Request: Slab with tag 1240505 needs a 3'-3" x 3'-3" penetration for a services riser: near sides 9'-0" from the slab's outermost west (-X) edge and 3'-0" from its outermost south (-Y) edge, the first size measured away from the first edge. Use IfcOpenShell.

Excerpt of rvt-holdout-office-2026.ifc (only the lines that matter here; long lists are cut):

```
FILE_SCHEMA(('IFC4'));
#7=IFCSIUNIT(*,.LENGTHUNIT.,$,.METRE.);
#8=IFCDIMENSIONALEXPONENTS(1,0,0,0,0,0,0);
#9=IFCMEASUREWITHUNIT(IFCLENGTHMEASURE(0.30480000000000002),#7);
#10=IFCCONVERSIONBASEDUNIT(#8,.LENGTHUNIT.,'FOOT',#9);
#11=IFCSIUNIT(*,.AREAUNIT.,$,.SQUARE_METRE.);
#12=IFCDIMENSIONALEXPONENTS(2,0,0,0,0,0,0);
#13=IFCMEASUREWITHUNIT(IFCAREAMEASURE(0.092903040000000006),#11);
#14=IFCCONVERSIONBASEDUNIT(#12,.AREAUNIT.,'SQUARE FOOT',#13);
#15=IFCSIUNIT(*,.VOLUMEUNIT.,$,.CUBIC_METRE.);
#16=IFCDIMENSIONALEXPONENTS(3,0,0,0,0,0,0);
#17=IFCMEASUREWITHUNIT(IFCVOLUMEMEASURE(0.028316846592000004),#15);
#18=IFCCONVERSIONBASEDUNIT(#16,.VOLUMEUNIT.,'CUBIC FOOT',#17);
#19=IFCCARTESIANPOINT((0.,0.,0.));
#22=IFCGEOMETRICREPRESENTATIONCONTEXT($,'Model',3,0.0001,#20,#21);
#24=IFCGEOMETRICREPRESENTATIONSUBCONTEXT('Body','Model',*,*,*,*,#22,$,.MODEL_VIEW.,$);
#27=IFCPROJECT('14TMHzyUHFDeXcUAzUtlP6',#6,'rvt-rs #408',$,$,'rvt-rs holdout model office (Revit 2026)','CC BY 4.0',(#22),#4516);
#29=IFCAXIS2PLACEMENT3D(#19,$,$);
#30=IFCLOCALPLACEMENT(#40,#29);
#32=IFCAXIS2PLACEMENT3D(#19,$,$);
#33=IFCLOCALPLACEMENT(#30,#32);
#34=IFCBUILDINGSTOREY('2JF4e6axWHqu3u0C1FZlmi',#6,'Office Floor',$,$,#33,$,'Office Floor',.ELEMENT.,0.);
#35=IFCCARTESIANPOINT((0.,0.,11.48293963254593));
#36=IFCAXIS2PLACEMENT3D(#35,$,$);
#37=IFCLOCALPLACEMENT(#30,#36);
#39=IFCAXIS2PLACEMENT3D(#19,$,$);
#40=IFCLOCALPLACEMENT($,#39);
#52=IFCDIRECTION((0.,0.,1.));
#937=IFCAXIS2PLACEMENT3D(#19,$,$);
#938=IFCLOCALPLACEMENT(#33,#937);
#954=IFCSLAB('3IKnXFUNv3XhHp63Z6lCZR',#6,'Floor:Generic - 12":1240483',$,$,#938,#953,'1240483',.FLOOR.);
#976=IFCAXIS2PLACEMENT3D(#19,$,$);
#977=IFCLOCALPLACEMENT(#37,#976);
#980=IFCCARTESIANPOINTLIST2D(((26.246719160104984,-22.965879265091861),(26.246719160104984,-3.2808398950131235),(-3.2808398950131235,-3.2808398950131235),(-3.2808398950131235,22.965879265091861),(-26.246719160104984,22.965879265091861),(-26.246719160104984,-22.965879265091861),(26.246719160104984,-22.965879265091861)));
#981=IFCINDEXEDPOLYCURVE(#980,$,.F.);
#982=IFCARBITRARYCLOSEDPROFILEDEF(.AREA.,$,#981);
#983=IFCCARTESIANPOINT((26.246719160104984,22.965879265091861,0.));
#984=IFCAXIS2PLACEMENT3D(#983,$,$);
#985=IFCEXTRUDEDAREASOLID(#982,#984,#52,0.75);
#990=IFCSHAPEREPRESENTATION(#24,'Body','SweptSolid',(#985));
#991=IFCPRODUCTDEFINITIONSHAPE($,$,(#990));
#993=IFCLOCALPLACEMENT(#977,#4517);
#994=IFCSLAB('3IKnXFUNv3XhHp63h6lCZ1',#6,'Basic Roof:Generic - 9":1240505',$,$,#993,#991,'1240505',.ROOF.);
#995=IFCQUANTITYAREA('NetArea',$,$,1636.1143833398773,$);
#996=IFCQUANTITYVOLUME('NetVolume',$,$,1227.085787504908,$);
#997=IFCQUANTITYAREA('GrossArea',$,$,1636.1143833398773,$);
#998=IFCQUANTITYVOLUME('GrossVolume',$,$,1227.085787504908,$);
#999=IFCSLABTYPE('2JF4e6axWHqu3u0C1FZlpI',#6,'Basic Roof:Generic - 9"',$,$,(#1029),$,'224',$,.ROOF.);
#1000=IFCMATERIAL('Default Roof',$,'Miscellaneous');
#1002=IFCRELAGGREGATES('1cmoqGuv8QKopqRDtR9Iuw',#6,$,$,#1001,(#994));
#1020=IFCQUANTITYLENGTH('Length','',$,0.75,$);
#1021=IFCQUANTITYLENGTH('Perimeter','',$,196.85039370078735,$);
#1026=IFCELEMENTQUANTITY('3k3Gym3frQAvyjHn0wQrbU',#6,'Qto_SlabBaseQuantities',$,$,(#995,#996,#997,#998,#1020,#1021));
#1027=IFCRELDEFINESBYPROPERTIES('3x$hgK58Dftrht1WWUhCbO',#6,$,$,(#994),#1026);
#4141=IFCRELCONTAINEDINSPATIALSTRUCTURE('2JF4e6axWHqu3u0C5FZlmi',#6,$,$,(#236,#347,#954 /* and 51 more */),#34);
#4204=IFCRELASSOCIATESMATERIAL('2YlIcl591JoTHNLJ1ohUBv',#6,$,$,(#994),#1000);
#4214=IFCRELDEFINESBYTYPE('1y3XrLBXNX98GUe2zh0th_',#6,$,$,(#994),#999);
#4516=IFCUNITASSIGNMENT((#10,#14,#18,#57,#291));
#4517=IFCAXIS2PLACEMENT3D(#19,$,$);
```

```python
import numpy as np
import ifcopenshell
import ifcopenshell.api.feature
import ifcopenshell.api.geometry
import ifcopenshell.api.pset
import ifcopenshell.api.root
import ifcopenshell.geom
import ifcopenshell.util.element
import ifcopenshell.util.placement
import ifcopenshell.util.representation
import ifcopenshell.util.shape
import ifcopenshell.util.unit

model = ifcopenshell.open("rvt-holdout-office-2026.ifc")
unit_scale = ifcopenshell.util.unit.calculate_unit_scale(model)
area_scale = ifcopenshell.util.unit.calculate_unit_scale(model, "AREAUNIT")
volume_scale = ifcopenshell.util.unit.calculate_unit_scale(model, "VOLUMEUNIT")
settings = ifcopenshell.geom.settings()


def volume(element):
    """Net volume in cubic metres, openings subtracted."""
    shape = ifcopenshell.geom.create_shape(settings, element)
    return ifcopenshell.util.shape.get_volume(shape.geometry)


slab = model.by_guid("3IKnXFUNv3XhHp63h6lCZ1")
before = volume(slab)

# Extent in the slab's own axes, in metres. The edges named are its -X and -Y sides.
slab_shape = ifcopenshell.geom.create_shape(settings, slab)
vertices = ifcopenshell.util.shape.get_vertices(slab_shape.geometry)
x_min, y_min, bottom = vertices.min(axis=0)
top = vertices[:, 2].max()

opening = ifcopenshell.api.root.create_entity(model, ifc_class="IfcOpeningElement", name="Services riser opening", predefined_type="OPENING")
context = ifcopenshell.util.representation.get_context(model, "Model", "Body", "MODEL_VIEW")
width, depth = 0.9906, 0.9906
outline = [(0.0, 0.0), (width, 0.0), (width, depth), (0.0, depth), (0.0, 0.0)]
# Overshoot both faces by 50 mm so the cut is clean.
shape = ifcopenshell.api.geometry.add_slab_representation(
    model, context=context, depth=top - bottom + 0.1, polyline=outline
)
ifcopenshell.api.geometry.assign_representation(model, product=opening, representation=shape)

matrix = ifcopenshell.util.placement.get_local_placement(slab.ObjectPlacement)
matrix[:, 3] = matrix @ np.append(np.array([x_min + 2.7432, y_min + 0.9144, bottom - 0.05]) / unit_scale, 1.0)
ifcopenshell.api.geometry.edit_object_placement(model, product=opening, matrix=matrix, is_si=False)
ifcopenshell.api.feature.add_feature(model, feature=opening, element=slab)

after = volume(slab)

# Update the slab's stored quantities.
qto = model.by_id(ifcopenshell.util.element.get_pset(slab, "Qto_SlabBaseQuantities", should_inherit=False)["id"])
ifcopenshell.api.pset.edit_qto(model, qto=qto, properties={
    "NetArea": after / (top - bottom) / area_scale,
    "NetVolume": after / volume_scale,
})

print(f"slab volume {before:.3f} -> {after:.3f} m3")

model.write("rvt-holdout-office-2026_v2.ifc")
```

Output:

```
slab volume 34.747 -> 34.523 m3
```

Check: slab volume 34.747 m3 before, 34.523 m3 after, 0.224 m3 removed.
